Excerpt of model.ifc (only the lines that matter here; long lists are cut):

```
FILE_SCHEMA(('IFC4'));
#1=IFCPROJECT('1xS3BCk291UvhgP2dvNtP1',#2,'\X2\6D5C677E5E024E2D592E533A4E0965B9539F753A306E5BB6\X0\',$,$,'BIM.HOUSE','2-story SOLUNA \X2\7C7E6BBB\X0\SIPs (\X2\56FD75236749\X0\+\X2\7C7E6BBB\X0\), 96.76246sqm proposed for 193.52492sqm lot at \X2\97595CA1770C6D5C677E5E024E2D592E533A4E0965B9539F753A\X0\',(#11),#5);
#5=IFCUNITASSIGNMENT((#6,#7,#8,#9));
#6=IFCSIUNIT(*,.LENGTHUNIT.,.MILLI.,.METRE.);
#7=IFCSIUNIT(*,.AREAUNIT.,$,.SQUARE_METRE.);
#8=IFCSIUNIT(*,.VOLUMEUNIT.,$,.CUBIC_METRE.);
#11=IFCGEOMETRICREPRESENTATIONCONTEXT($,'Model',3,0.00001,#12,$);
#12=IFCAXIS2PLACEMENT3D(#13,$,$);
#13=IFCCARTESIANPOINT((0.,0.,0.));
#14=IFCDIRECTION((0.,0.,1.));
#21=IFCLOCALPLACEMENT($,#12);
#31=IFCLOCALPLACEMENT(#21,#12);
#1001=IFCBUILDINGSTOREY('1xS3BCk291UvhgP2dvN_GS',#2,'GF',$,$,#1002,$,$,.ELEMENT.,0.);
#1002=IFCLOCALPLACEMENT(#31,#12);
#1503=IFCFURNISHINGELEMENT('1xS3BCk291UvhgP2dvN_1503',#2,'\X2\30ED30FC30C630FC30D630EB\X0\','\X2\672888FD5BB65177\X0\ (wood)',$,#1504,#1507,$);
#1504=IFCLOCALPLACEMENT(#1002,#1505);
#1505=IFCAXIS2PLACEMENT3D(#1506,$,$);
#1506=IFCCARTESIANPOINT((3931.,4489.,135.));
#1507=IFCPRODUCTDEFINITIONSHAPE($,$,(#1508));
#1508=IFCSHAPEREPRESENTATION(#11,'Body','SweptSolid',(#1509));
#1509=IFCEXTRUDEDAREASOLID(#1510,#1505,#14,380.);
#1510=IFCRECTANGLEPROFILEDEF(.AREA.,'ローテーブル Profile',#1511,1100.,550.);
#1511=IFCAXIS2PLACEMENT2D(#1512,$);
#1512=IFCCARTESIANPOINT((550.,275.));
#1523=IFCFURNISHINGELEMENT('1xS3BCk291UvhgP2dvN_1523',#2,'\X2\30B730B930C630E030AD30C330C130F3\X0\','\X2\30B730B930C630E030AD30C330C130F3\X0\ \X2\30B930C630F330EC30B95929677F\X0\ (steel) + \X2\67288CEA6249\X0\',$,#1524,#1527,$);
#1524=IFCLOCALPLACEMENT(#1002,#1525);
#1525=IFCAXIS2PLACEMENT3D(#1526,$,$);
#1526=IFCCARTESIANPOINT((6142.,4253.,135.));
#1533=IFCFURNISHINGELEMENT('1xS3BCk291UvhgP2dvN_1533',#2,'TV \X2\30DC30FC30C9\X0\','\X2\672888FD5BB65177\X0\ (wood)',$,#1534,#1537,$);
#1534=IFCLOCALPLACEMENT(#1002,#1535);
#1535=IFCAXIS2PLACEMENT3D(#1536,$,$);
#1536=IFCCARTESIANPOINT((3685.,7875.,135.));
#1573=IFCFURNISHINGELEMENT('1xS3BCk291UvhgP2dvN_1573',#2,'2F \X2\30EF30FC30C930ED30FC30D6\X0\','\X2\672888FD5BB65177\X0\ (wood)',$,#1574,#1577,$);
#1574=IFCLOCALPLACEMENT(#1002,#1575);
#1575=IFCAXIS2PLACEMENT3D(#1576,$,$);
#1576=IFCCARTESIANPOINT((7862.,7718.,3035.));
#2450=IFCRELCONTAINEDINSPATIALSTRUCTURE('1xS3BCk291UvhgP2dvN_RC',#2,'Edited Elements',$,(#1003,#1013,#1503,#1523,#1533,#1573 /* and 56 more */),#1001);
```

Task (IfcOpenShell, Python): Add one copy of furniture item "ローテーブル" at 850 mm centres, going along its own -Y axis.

```python
import ifcopenshell
import ifcopenshell.api.geometry
import ifcopenshell.api.root
import ifcopenshell.util.element
import ifcopenshell.util.placement

model = ifcopenshell.open("model.ifc")


def reuse_history(source, copy):
    """copy_class also copies each property set's owner history, people and application; keep the originals."""
    for rel in copy.IsDefinedBy:
        if rel.is_a("IfcRelDefinesByProperties") and (history := rel.RelatingPropertyDefinition.OwnerHistory):
            rel.RelatingPropertyDefinition.OwnerHistory = source.OwnerHistory
            ifcopenshell.util.element.remove_deep2(model, history)


source = model.by_guid("1xS3BCk291UvhgP2dvN_1503")
base = ifcopenshell.util.placement.get_local_placement(source.ObjectPlacement)
step = -base[:3, 1] * 850.0

for i in range(1, 2):
    copy = ifcopenshell.api.root.copy_class(model, product=source)
    copy.Representation = ifcopenshell.util.element.copy_deep(
        model, source.Representation, exclude=["IfcGeometricRepresentationContext", "IfcRepresentationMap"]
    )
    reuse_history(source, copy)
    matrix = base.copy()
    matrix[:3, 3] += i * step
    print("added at", matrix[:3, 3].round(3) + 0.0)
    ifcopenshell.api.geometry.edit_object_placement(model, product=copy, matrix=matrix, is_si=False)

model.write("model-out.ifc")
```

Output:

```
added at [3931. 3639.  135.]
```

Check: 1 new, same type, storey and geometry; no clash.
